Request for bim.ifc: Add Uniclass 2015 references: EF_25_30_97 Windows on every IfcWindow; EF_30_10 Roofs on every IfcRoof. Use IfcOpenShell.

First a look at what the model holds.

```python
import ifcopenshell

model = ifcopenshell.open("bim.ifc")
print(model.schema)
print("classifications:", [c.Name for c in model.by_type("IfcClassification")])
for ifc_class in ("IfcDoor", "IfcRoof", "IfcStair", "IfcWall", "IfcWindow"):
    print(ifc_class, len(model.by_type(ifc_class)))
```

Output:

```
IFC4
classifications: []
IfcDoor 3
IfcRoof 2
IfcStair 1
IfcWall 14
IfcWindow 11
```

```python
import ifcopenshell
import ifcopenshell.api.classification

model = ifcopenshell.open("bim.ifc")

system = ifcopenshell.api.classification.add_classification(model, classification="Uniclass 2015")

codes = {
    "IfcWindow": ("EF_25_30_97", "Windows"),
    "IfcRoof": ("EF_30_10", "Roofs"),
}
for ifc_class, (code, name) in codes.items():
    products = model.by_type(ifc_class)
    ifcopenshell.api.classification.add_reference(
        model, products=products, classification=system, identification=code, name=name
    )
    print(code, len(products))

model.write("bim_v2.ifc")
```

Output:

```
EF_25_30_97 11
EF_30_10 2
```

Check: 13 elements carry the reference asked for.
